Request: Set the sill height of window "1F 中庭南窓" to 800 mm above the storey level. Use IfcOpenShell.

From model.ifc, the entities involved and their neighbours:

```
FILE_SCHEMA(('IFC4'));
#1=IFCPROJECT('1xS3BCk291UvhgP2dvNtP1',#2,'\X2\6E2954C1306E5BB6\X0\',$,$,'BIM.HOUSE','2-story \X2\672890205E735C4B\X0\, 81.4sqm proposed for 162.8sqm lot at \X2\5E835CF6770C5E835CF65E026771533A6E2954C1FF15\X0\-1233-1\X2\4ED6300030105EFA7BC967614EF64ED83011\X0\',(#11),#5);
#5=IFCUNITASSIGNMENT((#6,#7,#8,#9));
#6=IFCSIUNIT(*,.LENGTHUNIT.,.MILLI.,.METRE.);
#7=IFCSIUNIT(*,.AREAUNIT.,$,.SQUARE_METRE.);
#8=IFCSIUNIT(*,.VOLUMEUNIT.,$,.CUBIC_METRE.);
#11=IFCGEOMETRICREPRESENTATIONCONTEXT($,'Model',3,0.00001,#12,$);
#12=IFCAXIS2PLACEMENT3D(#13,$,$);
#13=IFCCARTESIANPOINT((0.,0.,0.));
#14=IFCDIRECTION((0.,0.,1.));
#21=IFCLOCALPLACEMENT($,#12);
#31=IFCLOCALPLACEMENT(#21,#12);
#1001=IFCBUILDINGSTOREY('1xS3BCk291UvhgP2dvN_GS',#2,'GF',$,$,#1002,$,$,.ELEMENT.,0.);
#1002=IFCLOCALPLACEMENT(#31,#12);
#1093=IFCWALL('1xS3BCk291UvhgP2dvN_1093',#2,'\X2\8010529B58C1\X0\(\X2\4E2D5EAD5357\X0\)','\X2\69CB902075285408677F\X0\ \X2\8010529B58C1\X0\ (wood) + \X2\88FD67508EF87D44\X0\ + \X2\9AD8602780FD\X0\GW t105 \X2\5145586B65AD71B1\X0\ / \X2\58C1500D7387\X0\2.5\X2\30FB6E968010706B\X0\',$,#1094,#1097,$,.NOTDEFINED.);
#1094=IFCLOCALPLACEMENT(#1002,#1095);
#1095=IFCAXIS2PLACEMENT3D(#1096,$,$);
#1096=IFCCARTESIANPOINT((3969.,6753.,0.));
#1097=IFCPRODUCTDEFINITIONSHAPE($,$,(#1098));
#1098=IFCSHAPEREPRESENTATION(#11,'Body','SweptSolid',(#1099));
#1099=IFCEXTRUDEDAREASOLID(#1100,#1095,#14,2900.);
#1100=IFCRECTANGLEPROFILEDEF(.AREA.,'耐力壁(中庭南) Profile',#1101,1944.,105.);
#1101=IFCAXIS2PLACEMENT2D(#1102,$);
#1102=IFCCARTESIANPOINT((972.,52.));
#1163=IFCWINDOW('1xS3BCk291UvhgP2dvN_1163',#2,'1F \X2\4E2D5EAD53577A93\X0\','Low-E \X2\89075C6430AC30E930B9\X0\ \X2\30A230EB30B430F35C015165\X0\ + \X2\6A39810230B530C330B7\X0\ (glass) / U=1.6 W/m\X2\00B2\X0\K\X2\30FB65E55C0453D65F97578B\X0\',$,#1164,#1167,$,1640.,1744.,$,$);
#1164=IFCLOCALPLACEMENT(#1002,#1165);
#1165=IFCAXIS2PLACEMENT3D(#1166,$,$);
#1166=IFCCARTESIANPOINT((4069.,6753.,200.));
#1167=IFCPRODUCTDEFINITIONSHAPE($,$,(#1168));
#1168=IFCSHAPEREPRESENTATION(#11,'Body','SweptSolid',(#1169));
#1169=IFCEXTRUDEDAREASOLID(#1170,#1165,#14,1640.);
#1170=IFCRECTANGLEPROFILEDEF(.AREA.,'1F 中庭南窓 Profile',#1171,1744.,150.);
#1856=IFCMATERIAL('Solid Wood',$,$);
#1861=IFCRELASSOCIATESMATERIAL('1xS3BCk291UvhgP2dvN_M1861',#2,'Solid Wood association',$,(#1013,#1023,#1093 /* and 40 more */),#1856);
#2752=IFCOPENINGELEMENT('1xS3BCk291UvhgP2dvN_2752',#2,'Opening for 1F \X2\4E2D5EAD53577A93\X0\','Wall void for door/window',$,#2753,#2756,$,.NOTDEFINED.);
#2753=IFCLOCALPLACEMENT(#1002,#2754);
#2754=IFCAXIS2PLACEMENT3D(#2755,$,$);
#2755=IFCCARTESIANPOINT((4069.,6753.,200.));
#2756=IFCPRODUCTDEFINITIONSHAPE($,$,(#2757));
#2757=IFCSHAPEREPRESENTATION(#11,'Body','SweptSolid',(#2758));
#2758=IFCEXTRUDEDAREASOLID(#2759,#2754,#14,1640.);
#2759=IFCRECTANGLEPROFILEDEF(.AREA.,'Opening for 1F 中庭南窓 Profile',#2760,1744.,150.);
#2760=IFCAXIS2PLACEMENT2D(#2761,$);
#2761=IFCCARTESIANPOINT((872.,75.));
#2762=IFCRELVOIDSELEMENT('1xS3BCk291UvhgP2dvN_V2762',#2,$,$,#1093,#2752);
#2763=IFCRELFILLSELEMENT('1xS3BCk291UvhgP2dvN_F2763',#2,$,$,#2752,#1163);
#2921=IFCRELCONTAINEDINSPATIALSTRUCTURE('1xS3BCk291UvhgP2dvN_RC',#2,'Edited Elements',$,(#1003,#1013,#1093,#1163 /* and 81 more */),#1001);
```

```python
import numpy as np
import ifcopenshell
import ifcopenshell.api.geometry
import ifcopenshell.geom
import ifcopenshell.util.element
import ifcopenshell.util.placement
import ifcopenshell.util.shape
import ifcopenshell.util.unit

model = ifcopenshell.open("model.ifc")
unit_scale = ifcopenshell.util.unit.calculate_unit_scale(model)

window = model.by_id(1163)
opening = window.FillsVoids[0].RelatingOpeningElement
storey = ifcopenshell.util.element.get_container(window, ifc_class="IfcBuildingStorey")
level = ifcopenshell.util.placement.get_local_placement(storey.ObjectPlacement)[2, 3]

# The opening's origin need not be at the sill, so measure its lowest point.
shape = ifcopenshell.geom.create_shape(ifcopenshell.geom.settings(), opening)
bottom = ifcopenshell.util.shape.get_shape_bottom_elevation(shape, shape.geometry) / unit_scale
dz = level + 0.8 / unit_scale - bottom

shift = np.array([0.0, 0.0, dz])
# The window is not placed relative to its opening, so move both.
for product in (opening, window):
    matrix = ifcopenshell.util.placement.get_local_placement(product.ObjectPlacement)
    matrix[:3, 3] += shift
    ifcopenshell.api.geometry.edit_object_placement(model, product=product, matrix=matrix, is_si=False)

print(f"moved by {dz * unit_scale:+.3f} m")

model.write("model_edited.ifc")
```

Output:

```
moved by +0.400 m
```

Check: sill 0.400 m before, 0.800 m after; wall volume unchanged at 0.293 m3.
